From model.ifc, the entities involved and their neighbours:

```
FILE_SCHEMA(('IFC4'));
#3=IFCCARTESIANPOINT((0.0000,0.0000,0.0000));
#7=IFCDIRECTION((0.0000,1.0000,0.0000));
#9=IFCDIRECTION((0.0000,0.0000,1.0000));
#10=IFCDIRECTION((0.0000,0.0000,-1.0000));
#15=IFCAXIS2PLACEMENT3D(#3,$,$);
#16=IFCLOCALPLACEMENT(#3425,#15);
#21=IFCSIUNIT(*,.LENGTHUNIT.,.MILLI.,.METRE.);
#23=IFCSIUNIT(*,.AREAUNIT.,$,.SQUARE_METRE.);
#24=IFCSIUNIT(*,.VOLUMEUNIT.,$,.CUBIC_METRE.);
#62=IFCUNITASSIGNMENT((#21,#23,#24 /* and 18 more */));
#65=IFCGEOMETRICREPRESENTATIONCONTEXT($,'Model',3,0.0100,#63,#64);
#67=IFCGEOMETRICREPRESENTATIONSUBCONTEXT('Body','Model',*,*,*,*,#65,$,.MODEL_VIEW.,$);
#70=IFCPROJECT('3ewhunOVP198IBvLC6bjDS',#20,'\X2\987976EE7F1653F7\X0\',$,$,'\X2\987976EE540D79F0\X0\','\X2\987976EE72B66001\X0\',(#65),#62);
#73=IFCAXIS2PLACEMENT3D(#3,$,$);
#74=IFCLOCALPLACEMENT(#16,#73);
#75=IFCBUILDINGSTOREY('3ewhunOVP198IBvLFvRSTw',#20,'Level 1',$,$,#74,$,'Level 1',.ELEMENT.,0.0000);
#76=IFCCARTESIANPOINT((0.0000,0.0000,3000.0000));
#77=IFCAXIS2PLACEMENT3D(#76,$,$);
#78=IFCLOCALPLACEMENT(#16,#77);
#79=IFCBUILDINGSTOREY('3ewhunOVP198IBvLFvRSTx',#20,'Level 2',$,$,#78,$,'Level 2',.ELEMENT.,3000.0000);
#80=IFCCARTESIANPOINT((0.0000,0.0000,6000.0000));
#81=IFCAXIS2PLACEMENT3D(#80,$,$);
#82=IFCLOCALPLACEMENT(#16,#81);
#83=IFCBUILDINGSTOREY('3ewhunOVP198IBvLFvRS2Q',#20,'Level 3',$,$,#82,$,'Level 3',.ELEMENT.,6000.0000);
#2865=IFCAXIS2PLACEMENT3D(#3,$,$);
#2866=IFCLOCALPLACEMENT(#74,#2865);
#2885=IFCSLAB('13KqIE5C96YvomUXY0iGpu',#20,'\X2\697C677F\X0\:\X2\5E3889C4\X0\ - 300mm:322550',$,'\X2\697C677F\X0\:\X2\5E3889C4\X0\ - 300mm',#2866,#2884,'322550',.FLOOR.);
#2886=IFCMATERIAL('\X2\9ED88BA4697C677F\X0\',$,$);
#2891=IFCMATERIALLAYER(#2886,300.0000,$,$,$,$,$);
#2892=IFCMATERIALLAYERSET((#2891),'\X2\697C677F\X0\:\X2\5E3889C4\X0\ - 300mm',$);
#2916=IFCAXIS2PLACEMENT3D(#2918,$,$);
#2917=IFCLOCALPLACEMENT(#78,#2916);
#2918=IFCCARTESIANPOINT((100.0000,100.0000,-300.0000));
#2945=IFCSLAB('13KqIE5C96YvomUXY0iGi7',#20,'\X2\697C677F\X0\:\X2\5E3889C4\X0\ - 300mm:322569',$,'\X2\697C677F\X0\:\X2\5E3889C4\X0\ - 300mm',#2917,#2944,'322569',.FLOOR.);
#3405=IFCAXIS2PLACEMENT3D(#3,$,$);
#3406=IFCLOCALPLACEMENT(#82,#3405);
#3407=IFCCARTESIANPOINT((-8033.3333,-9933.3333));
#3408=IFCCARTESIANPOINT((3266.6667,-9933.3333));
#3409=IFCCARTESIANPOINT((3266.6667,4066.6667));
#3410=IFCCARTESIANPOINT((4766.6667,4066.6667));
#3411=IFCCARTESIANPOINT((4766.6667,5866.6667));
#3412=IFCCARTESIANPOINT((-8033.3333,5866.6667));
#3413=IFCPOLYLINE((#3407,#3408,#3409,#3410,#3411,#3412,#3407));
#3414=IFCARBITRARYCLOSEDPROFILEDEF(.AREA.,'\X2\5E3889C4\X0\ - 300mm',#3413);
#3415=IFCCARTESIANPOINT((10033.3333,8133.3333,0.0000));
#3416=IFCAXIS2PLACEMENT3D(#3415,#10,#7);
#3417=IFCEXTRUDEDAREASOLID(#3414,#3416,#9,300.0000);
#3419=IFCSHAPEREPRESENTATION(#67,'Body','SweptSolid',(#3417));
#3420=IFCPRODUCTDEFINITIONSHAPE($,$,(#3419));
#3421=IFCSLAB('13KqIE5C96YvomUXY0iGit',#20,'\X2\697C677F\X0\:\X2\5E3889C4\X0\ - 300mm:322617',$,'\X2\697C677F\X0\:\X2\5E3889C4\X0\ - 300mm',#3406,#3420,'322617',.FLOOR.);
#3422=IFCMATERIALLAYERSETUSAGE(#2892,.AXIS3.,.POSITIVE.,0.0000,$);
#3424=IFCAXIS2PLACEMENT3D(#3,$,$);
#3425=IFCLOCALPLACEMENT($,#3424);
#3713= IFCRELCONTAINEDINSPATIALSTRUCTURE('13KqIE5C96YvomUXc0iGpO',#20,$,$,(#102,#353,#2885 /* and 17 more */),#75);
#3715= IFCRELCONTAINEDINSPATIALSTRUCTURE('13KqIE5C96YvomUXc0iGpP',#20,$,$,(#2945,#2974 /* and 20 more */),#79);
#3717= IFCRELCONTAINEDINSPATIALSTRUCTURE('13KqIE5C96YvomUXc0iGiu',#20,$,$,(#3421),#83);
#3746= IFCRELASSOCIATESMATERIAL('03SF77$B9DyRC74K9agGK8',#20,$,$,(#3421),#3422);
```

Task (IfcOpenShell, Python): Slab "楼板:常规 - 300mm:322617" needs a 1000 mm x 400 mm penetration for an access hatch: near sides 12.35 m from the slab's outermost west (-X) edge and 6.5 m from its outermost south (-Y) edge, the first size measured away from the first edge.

```python
import numpy as np
import ifcopenshell
import ifcopenshell.api.feature
import ifcopenshell.api.geometry
import ifcopenshell.api.root
import ifcopenshell.geom
import ifcopenshell.util.placement
import ifcopenshell.util.representation
import ifcopenshell.util.shape
import ifcopenshell.util.unit

model = ifcopenshell.open("model.ifc")
unit_scale = ifcopenshell.util.unit.calculate_unit_scale(model)
settings = ifcopenshell.geom.settings()


def volume(element):
    """Net volume in cubic metres, openings subtracted."""
    shape = ifcopenshell.geom.create_shape(settings, element)
    return ifcopenshell.util.shape.get_volume(shape.geometry)


slab = model.by_guid("13KqIE5C96YvomUXY0iGit")
before = volume(slab)

# Extent in the slab's own axes, in metres. The edges named are its -X and -Y sides.
slab_shape = ifcopenshell.geom.create_shape(settings, slab)
vertices = ifcopenshell.util.shape.get_vertices(slab_shape.geometry)
x_min, y_min, bottom = vertices.min(axis=0)
top = vertices[:, 2].max()

opening = ifcopenshell.api.root.create_entity(model, ifc_class="IfcOpeningElement", name="Access hatch opening", predefined_type="OPENING")
context = ifcopenshell.util.representation.get_context(model, "Model", "Body", "MODEL_VIEW")
width, depth = 1, 0.4
outline = [(0.0, 0.0), (width, 0.0), (width, depth), (0.0, depth), (0.0, 0.0)]
# Overshoot both faces by 50 mm so the cut is clean.
shape = ifcopenshell.api.geometry.add_slab_representation(
    model, context=context, depth=top - bottom + 0.1, polyline=outline
)
ifcopenshell.api.geometry.assign_representation(model, product=opening, representation=shape)

matrix = ifcopenshell.util.placement.get_local_placement(slab.ObjectPlacement)
matrix[:, 3] = matrix @ np.append(np.array([x_min + 12.35, y_min + 6.5, bottom - 0.05]) / unit_scale, 1.0)
ifcopenshell.api.geometry.edit_object_placement(model, product=opening, matrix=matrix, is_si=False)
ifcopenshell.api.feature.add_feature(model, feature=opening, element=slab)

after = volume(slab)

print(f"slab volume {before:.3f} -> {after:.3f} m3")

model.write("model_updated.ifc")
```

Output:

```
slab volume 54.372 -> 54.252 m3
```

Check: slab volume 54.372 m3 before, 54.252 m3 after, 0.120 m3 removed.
